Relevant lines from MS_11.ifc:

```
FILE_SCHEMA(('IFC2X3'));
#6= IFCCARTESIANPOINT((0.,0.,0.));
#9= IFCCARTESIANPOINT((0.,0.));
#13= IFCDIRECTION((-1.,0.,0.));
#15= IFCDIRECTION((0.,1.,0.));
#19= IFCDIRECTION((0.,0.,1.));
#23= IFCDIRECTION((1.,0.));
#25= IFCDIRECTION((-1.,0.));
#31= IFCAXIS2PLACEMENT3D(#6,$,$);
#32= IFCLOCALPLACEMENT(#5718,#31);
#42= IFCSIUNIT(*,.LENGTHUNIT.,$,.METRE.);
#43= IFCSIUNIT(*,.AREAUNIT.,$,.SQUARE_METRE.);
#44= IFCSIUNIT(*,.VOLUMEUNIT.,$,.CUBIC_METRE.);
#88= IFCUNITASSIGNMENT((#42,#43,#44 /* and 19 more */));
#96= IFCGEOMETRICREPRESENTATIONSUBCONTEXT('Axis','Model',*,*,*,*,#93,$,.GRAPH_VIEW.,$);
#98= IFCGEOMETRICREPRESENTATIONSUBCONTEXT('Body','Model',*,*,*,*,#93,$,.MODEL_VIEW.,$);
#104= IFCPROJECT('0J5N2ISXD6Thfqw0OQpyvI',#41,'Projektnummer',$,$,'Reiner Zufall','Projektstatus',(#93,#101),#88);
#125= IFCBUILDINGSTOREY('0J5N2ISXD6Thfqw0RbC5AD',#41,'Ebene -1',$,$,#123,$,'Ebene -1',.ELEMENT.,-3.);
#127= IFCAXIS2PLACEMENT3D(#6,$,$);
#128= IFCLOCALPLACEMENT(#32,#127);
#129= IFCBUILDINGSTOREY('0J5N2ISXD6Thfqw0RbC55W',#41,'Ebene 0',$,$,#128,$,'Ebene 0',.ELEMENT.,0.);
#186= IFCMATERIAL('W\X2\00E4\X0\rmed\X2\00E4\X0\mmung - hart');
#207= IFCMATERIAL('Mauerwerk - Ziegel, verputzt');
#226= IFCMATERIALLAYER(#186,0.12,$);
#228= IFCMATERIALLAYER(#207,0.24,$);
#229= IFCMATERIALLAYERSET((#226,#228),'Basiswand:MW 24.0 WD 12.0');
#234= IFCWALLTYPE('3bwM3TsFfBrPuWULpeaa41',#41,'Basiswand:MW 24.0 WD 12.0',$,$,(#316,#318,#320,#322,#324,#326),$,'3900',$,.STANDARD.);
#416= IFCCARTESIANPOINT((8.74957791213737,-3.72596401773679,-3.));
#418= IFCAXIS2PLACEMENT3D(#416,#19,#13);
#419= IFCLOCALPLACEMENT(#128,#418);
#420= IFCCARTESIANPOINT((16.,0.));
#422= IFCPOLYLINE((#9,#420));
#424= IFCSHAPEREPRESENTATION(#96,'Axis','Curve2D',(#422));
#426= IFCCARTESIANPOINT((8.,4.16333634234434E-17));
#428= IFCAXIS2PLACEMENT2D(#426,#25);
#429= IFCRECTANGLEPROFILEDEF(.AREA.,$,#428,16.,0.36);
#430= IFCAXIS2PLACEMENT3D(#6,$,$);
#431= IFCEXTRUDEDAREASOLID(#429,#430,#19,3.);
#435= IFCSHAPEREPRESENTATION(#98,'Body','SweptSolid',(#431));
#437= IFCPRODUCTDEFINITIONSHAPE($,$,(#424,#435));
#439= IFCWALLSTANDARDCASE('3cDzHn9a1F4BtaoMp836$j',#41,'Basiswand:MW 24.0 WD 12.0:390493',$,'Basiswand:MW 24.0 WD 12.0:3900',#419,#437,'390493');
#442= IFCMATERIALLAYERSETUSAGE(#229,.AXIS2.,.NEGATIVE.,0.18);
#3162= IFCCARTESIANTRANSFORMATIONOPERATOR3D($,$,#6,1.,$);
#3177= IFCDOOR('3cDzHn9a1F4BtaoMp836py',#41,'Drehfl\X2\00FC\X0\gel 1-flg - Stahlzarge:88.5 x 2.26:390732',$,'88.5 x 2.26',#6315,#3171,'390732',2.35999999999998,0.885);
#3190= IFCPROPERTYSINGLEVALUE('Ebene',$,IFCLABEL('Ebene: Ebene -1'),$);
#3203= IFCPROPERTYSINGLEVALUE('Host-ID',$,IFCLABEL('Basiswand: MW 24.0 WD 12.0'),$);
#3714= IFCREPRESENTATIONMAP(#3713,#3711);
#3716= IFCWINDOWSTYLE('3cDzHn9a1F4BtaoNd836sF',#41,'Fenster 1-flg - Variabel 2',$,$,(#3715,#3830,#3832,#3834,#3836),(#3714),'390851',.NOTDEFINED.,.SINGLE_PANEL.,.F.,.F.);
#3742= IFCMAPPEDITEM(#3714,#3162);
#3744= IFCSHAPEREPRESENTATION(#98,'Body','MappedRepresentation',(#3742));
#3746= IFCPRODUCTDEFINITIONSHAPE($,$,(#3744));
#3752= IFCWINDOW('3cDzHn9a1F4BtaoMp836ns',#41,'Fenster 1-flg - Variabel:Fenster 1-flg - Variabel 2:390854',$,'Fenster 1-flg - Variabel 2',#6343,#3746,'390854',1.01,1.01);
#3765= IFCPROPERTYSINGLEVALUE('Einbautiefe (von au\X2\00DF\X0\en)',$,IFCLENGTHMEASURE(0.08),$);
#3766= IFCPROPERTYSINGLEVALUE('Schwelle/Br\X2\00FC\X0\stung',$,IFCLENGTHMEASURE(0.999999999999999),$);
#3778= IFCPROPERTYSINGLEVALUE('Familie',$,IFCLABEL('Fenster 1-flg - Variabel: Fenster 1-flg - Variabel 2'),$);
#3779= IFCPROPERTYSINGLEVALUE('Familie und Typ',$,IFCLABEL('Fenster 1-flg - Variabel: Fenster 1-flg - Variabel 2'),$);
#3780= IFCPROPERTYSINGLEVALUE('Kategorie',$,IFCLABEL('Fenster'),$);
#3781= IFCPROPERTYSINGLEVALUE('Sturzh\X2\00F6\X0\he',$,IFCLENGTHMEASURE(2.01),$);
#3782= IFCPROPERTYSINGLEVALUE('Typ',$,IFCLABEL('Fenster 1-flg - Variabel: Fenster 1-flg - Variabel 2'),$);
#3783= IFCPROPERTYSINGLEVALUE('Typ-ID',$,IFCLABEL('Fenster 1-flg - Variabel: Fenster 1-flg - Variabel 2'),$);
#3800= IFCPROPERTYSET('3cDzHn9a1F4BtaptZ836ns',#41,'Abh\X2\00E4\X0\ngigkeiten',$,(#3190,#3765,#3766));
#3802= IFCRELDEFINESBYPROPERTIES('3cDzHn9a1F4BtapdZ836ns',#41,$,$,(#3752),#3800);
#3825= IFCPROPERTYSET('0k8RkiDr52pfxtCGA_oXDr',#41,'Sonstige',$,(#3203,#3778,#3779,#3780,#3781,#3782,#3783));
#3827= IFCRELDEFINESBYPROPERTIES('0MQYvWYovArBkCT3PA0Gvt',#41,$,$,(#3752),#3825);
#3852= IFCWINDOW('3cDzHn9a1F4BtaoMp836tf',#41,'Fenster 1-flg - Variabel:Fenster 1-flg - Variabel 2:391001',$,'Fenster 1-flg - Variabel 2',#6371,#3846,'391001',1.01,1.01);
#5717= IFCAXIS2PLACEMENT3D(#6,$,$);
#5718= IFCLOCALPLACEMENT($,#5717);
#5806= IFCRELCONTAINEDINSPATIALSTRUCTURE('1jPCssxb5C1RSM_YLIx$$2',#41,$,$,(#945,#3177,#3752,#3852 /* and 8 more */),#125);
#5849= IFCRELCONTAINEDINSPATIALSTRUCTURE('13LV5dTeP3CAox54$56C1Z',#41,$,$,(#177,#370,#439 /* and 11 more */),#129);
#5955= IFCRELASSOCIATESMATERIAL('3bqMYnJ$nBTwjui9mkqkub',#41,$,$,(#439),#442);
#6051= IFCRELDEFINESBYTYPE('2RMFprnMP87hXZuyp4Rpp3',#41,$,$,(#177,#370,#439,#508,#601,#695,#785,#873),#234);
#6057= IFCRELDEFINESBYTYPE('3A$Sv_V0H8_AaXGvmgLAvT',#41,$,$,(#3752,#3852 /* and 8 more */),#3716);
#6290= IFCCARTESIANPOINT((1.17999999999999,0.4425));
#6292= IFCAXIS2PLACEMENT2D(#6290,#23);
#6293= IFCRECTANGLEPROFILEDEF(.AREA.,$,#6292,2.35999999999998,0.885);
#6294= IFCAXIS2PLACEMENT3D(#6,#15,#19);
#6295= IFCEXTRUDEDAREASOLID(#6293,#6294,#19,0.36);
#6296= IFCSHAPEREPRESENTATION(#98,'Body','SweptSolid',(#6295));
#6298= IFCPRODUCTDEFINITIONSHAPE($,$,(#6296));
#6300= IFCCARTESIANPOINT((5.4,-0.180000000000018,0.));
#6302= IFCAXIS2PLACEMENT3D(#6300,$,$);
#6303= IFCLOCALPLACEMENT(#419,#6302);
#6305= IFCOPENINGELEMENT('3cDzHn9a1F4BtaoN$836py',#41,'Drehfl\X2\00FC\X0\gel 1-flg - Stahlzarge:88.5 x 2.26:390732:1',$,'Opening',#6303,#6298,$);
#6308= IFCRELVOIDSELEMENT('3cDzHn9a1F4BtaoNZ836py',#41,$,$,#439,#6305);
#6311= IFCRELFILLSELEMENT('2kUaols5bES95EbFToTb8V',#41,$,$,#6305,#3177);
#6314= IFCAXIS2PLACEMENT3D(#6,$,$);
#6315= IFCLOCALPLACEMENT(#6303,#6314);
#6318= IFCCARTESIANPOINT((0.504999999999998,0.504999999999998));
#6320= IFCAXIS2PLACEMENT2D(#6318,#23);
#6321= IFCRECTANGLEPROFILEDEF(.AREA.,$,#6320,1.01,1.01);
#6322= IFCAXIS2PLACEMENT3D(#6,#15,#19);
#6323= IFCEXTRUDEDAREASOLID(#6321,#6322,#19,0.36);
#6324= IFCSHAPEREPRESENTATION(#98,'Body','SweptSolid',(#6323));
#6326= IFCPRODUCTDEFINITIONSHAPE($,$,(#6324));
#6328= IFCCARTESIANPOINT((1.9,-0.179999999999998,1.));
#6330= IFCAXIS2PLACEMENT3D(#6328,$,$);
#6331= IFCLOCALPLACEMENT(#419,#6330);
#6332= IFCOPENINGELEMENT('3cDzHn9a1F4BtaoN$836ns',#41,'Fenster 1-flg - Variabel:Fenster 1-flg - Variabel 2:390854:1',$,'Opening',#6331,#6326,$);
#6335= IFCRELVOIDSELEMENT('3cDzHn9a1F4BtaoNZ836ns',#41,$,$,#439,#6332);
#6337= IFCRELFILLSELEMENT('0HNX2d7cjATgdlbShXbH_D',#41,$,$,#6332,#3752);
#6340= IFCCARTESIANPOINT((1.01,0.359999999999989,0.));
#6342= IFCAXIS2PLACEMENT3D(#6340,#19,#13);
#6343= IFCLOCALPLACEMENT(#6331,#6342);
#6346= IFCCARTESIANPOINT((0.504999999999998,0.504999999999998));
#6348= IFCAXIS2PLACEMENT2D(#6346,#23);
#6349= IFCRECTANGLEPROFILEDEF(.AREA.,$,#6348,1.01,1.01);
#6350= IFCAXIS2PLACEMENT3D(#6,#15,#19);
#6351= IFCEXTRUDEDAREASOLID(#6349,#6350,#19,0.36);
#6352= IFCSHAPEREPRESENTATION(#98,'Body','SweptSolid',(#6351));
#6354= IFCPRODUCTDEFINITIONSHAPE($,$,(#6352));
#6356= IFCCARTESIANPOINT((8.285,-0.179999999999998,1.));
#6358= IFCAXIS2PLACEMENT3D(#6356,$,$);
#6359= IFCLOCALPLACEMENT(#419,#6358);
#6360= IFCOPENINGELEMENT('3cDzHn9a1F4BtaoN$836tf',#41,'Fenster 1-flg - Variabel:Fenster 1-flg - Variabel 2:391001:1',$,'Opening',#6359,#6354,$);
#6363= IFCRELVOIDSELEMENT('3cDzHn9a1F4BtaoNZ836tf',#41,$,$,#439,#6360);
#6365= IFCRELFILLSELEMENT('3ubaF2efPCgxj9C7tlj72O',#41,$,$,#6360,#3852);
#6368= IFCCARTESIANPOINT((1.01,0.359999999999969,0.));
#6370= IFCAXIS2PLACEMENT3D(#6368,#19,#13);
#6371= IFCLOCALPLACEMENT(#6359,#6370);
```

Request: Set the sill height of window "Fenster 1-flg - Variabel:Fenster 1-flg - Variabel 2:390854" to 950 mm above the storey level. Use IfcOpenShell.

```python
import numpy as np
import ifcopenshell
import ifcopenshell.api.geometry
import ifcopenshell.api.pset
import ifcopenshell.geom
import ifcopenshell.util.element
import ifcopenshell.util.placement
import ifcopenshell.util.shape
import ifcopenshell.util.unit

model = ifcopenshell.open("MS_11.ifc")
unit_scale = ifcopenshell.util.unit.calculate_unit_scale(model)

window = model.by_guid("3cDzHn9a1F4BtaoMp836ns")
opening = window.FillsVoids[0].RelatingOpeningElement
storey = ifcopenshell.util.element.get_container(window, ifc_class="IfcBuildingStorey")
level = ifcopenshell.util.placement.get_local_placement(storey.ObjectPlacement)[2, 3]

# The opening's origin need not be at the sill, so measure its lowest point.
shape = ifcopenshell.geom.create_shape(ifcopenshell.geom.settings(), opening)
bottom = ifcopenshell.util.shape.get_shape_bottom_elevation(shape, shape.geometry) / unit_scale
dz = level + 0.95 - bottom

shift = np.array([0.0, 0.0, dz])
# The window is placed relative to its opening, so it follows when the opening moves.
matrix = ifcopenshell.util.placement.get_local_placement(opening.ObjectPlacement)
matrix[:3, 3] += shift
ifcopenshell.api.geometry.edit_object_placement(
    model, product=opening, matrix=matrix, is_si=False, should_transform_children=True
)

# Keep the stored heights in step.
pset = model.by_id(ifcopenshell.util.element.get_pset(window, "Abhängigkeiten", should_inherit=False)["id"])
ifcopenshell.api.pset.edit_pset(model, pset=pset, properties={
    "Schwelle/Brüstung": model.create_entity("IfcLengthMeasure", ifcopenshell.util.element.get_pset(window, "Abhängigkeiten", "Schwelle/Brüstung") + dz),
})
pset = model.by_id(ifcopenshell.util.element.get_pset(window, "Sonstige", should_inherit=False)["id"])
ifcopenshell.api.pset.edit_pset(model, pset=pset, properties={
    "Sturzhöhe": model.create_entity("IfcLengthMeasure", ifcopenshell.util.element.get_pset(window, "Sonstige", "Sturzhöhe") + dz),
})

print(f"moved by {dz * unit_scale:+.3f} m")

model.write("MS_11_edited.ifc")
```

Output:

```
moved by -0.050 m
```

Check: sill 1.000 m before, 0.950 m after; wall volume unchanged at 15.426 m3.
